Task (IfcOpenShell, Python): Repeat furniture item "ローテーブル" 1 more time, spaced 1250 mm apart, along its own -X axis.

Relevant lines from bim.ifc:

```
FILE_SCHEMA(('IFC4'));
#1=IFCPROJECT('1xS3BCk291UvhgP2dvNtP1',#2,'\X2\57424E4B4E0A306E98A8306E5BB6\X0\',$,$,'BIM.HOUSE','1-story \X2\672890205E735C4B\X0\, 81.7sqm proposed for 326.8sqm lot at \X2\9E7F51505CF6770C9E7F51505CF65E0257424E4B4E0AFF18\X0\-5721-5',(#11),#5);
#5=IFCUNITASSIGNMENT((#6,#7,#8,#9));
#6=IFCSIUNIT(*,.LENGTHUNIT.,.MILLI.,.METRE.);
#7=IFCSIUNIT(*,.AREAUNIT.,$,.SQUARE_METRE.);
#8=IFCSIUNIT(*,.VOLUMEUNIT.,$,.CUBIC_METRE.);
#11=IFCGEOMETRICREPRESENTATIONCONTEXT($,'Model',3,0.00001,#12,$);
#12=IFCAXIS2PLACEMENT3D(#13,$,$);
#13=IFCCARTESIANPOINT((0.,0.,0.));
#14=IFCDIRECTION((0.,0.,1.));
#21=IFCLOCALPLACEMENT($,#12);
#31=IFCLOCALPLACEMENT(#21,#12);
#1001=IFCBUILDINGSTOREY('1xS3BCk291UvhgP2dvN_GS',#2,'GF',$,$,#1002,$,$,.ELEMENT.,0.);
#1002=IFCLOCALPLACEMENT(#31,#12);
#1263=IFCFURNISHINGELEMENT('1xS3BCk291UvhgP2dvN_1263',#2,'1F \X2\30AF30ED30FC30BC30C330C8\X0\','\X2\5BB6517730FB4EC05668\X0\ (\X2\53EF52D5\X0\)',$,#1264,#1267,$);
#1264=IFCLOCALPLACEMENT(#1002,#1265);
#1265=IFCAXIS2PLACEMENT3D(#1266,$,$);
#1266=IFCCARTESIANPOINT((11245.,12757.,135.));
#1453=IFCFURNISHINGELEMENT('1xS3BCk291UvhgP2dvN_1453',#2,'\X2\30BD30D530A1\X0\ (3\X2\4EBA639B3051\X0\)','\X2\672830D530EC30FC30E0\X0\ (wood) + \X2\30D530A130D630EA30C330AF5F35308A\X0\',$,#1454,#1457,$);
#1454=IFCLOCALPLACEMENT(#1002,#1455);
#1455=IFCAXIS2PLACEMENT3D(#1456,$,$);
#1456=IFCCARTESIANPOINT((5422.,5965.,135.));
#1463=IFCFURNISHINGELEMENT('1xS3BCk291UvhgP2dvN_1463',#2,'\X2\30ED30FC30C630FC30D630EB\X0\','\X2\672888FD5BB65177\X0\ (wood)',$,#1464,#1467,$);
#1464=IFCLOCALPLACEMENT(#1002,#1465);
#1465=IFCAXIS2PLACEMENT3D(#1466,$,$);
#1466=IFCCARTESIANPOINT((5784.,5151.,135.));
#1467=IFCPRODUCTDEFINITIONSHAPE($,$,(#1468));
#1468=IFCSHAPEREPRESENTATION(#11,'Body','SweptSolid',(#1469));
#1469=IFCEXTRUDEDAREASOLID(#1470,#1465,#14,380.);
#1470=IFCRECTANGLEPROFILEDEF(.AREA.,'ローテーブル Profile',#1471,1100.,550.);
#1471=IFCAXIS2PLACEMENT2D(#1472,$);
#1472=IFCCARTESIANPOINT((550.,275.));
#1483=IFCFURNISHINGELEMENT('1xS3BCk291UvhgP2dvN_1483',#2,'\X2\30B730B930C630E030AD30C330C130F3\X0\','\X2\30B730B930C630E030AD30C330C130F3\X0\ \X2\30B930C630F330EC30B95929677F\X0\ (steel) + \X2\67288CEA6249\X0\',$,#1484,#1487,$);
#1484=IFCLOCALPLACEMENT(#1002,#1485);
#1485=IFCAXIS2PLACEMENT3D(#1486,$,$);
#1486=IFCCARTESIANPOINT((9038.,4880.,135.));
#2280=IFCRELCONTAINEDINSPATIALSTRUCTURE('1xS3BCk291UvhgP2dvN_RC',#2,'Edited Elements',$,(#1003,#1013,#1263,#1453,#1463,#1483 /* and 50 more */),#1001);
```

```python
import ifcopenshell
import ifcopenshell.api.geometry
import ifcopenshell.api.root
import ifcopenshell.util.element
import ifcopenshell.util.placement

model = ifcopenshell.open("bim.ifc")


def reuse_history(source, copy):
    """copy_class also copies each property set's owner history, people and application; keep the originals."""
    for rel in copy.IsDefinedBy:
        if rel.is_a("IfcRelDefinesByProperties") and (history := rel.RelatingPropertyDefinition.OwnerHistory):
            rel.RelatingPropertyDefinition.OwnerHistory = source.OwnerHistory
            ifcopenshell.util.element.remove_deep2(model, history)


source = model.by_id(1463)
base = ifcopenshell.util.placement.get_local_placement(source.ObjectPlacement)
step = -base[:3, 0] * 1250.0

for i in range(1, 2):
    copy = ifcopenshell.api.root.copy_class(model, product=source)
    copy.Representation = ifcopenshell.util.element.copy_deep(
        model, source.Representation, exclude=["IfcGeometricRepresentationContext", "IfcRepresentationMap"]
    )
    reuse_history(source, copy)
    matrix = base.copy()
    matrix[:3, 3] += i * step
    print("added at", matrix[:3, 3].round(3) + 0.0)
    ifcopenshell.api.geometry.edit_object_placement(model, product=copy, matrix=matrix, is_si=False)

model.write("bim_edited.ifc")
```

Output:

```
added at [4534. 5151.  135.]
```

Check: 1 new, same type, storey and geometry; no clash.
